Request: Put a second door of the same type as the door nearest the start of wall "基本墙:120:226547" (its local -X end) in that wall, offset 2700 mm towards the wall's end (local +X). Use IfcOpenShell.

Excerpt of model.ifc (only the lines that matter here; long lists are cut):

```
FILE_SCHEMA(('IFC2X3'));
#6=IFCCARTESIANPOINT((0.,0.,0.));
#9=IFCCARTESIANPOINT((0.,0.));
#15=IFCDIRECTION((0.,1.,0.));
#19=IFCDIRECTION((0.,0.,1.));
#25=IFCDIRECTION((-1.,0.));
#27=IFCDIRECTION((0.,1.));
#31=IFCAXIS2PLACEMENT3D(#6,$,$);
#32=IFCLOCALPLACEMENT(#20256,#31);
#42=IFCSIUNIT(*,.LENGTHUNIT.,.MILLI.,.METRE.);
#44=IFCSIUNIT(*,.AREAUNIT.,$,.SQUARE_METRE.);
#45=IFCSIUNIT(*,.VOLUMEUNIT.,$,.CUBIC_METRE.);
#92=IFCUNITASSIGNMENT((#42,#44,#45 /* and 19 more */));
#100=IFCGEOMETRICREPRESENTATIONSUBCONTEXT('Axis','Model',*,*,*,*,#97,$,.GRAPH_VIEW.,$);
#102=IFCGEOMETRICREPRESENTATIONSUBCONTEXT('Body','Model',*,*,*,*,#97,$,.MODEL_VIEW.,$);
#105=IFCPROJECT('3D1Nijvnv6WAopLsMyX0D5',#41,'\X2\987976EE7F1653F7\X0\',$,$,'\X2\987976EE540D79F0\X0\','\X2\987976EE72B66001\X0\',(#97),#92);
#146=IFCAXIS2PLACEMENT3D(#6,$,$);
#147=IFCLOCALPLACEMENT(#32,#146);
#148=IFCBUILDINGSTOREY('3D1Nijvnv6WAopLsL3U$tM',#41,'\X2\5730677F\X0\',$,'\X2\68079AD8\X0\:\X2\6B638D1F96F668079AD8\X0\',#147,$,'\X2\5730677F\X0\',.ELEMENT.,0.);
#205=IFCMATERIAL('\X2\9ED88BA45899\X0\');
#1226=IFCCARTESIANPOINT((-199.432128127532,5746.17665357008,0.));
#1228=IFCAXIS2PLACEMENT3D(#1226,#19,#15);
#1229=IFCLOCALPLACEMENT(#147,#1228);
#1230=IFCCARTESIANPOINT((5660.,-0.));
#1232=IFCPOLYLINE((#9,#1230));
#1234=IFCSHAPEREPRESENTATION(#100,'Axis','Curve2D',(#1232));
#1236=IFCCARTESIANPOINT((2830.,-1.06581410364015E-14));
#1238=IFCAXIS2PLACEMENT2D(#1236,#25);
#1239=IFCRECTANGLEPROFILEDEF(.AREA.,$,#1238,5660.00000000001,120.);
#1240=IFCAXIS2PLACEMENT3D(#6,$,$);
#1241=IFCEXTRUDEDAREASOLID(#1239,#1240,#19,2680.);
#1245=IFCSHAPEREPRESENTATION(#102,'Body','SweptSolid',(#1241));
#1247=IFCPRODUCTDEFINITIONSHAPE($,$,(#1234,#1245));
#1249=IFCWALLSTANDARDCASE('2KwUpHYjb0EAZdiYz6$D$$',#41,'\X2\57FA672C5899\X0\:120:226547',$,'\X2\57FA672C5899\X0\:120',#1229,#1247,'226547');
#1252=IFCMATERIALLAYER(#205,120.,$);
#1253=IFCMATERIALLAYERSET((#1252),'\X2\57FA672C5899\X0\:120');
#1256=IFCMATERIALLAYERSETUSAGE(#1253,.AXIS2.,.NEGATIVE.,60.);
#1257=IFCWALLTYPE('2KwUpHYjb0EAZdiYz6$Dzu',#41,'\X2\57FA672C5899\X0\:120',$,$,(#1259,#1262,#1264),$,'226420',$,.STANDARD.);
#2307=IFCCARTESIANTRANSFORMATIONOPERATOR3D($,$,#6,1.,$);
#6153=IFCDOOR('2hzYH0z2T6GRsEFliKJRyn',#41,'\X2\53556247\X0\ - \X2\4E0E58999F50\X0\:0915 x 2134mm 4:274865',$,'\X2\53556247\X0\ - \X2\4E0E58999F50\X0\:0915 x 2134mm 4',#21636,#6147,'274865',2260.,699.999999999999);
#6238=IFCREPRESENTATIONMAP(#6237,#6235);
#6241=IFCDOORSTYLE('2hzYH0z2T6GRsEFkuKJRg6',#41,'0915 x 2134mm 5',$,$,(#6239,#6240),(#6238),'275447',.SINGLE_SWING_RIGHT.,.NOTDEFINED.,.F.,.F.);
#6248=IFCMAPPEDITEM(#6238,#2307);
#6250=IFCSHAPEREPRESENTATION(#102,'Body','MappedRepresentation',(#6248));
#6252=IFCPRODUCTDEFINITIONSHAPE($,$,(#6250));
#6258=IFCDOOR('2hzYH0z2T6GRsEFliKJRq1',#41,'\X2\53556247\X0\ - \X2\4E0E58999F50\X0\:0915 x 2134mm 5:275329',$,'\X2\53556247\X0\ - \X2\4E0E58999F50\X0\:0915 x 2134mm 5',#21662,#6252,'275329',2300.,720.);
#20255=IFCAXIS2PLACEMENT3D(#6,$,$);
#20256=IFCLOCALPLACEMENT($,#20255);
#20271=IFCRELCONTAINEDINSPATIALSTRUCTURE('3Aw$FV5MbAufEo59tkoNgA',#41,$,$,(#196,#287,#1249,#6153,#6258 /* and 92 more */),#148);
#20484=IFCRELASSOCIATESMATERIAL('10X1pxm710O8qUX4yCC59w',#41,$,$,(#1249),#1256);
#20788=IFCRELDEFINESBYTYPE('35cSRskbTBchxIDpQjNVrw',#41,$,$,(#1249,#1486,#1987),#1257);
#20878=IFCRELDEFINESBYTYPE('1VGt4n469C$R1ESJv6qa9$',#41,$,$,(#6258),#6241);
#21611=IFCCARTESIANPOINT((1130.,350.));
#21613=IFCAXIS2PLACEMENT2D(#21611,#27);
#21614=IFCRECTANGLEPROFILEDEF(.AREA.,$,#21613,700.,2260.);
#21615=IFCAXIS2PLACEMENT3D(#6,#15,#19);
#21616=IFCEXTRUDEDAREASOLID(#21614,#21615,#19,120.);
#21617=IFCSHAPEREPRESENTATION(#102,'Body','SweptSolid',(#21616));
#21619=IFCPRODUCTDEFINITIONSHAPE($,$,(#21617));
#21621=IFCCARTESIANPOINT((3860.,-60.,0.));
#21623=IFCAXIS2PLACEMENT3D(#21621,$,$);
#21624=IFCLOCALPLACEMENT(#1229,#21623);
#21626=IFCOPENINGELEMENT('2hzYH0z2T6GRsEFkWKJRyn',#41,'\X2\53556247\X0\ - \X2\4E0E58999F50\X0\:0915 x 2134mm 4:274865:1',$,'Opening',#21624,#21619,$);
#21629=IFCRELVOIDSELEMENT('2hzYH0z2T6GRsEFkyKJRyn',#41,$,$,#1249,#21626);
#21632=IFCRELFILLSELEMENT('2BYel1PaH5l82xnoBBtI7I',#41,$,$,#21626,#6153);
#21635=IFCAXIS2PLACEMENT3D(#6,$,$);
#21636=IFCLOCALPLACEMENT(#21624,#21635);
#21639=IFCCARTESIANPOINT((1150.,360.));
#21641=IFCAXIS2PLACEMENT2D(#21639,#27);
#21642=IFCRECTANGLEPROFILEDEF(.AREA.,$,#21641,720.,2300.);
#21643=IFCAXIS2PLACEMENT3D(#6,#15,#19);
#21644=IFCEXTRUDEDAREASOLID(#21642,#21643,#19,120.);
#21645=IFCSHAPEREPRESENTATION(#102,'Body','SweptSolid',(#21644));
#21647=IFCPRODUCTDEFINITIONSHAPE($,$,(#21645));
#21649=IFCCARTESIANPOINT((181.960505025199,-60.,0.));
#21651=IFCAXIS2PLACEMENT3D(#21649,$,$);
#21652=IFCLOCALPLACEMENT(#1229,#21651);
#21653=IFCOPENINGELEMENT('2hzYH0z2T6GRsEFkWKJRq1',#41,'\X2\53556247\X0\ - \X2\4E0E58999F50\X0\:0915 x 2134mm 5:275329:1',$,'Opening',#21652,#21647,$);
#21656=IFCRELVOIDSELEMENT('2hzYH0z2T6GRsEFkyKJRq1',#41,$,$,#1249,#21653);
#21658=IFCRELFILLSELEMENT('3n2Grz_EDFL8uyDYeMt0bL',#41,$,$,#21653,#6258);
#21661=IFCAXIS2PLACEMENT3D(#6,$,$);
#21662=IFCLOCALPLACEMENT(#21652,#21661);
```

```python
import ifcopenshell
import ifcopenshell.api.feature
import ifcopenshell.api.geometry
import ifcopenshell.api.root
import ifcopenshell.geom
import ifcopenshell.util.element
import ifcopenshell.util.placement
import ifcopenshell.util.shape

model = ifcopenshell.open("model.ifc")
settings = ifcopenshell.geom.settings()


def volume(element):
    """Net volume in cubic metres, openings subtracted."""
    shape = ifcopenshell.geom.create_shape(settings, element)
    return ifcopenshell.util.shape.get_volume(shape.geometry)


def reuse_history(source, copy):
    """copy_class also copies each property set's owner history, people and application; keep the originals."""
    for rel in copy.IsDefinedBy:
        if rel.is_a("IfcRelDefinesByProperties") and (history := rel.RelatingPropertyDefinition.OwnerHistory):
            rel.RelatingPropertyDefinition.OwnerHistory = source.OwnerHistory
            ifcopenshell.util.element.remove_deep2(model, history)


door = model.by_guid("2hzYH0z2T6GRsEFliKJRq1")
opening = door.FillsVoids[0].RelatingOpeningElement
wall = opening.VoidsElements[0].RelatingBuildingElement
before = volume(wall)
shift = ifcopenshell.util.placement.get_local_placement(wall.ObjectPlacement)[:3, 0] * 2700.0

# copy_class copies the void relationship, type, container and properties, but no geometry.
new_opening = ifcopenshell.api.root.copy_class(model, product=opening)
new_opening.Representation = ifcopenshell.util.element.copy_deep(
    model, opening.Representation, exclude=["IfcGeometricRepresentationContext", "IfcRepresentationMap"]
)
new_opening.Name = "单扇 - 与墙齐:0915 x 2134mm 5"
new_door = ifcopenshell.api.root.copy_class(model, product=door)
new_door.Representation = ifcopenshell.util.element.copy_deep(
    model, door.Representation, exclude=["IfcGeometricRepresentationContext", "IfcRepresentationMap"]
)
new_door.Name = "单扇 - 与墙齐:0915 x 2134mm 5"
new_door.Tag = None
reuse_history(door, new_door)
fills = ifcopenshell.api.feature.add_filling(model, opening=new_opening, element=new_door)
fills.OwnerHistory = new_door.OwnerHistory  # required in IFC2X3

for old, new in ((opening, new_opening), (door, new_door)):
    matrix = ifcopenshell.util.placement.get_local_placement(old.ObjectPlacement)
    matrix[:3, 3] += shift
    ifcopenshell.api.geometry.edit_object_placement(model, product=new, matrix=matrix, is_si=False)

after = volume(wall)

print(f"wall volume {before:.3f} -> {after:.3f} m3")

model.write("model-out.ifc")
```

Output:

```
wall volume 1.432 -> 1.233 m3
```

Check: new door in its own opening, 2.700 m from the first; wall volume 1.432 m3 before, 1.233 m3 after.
